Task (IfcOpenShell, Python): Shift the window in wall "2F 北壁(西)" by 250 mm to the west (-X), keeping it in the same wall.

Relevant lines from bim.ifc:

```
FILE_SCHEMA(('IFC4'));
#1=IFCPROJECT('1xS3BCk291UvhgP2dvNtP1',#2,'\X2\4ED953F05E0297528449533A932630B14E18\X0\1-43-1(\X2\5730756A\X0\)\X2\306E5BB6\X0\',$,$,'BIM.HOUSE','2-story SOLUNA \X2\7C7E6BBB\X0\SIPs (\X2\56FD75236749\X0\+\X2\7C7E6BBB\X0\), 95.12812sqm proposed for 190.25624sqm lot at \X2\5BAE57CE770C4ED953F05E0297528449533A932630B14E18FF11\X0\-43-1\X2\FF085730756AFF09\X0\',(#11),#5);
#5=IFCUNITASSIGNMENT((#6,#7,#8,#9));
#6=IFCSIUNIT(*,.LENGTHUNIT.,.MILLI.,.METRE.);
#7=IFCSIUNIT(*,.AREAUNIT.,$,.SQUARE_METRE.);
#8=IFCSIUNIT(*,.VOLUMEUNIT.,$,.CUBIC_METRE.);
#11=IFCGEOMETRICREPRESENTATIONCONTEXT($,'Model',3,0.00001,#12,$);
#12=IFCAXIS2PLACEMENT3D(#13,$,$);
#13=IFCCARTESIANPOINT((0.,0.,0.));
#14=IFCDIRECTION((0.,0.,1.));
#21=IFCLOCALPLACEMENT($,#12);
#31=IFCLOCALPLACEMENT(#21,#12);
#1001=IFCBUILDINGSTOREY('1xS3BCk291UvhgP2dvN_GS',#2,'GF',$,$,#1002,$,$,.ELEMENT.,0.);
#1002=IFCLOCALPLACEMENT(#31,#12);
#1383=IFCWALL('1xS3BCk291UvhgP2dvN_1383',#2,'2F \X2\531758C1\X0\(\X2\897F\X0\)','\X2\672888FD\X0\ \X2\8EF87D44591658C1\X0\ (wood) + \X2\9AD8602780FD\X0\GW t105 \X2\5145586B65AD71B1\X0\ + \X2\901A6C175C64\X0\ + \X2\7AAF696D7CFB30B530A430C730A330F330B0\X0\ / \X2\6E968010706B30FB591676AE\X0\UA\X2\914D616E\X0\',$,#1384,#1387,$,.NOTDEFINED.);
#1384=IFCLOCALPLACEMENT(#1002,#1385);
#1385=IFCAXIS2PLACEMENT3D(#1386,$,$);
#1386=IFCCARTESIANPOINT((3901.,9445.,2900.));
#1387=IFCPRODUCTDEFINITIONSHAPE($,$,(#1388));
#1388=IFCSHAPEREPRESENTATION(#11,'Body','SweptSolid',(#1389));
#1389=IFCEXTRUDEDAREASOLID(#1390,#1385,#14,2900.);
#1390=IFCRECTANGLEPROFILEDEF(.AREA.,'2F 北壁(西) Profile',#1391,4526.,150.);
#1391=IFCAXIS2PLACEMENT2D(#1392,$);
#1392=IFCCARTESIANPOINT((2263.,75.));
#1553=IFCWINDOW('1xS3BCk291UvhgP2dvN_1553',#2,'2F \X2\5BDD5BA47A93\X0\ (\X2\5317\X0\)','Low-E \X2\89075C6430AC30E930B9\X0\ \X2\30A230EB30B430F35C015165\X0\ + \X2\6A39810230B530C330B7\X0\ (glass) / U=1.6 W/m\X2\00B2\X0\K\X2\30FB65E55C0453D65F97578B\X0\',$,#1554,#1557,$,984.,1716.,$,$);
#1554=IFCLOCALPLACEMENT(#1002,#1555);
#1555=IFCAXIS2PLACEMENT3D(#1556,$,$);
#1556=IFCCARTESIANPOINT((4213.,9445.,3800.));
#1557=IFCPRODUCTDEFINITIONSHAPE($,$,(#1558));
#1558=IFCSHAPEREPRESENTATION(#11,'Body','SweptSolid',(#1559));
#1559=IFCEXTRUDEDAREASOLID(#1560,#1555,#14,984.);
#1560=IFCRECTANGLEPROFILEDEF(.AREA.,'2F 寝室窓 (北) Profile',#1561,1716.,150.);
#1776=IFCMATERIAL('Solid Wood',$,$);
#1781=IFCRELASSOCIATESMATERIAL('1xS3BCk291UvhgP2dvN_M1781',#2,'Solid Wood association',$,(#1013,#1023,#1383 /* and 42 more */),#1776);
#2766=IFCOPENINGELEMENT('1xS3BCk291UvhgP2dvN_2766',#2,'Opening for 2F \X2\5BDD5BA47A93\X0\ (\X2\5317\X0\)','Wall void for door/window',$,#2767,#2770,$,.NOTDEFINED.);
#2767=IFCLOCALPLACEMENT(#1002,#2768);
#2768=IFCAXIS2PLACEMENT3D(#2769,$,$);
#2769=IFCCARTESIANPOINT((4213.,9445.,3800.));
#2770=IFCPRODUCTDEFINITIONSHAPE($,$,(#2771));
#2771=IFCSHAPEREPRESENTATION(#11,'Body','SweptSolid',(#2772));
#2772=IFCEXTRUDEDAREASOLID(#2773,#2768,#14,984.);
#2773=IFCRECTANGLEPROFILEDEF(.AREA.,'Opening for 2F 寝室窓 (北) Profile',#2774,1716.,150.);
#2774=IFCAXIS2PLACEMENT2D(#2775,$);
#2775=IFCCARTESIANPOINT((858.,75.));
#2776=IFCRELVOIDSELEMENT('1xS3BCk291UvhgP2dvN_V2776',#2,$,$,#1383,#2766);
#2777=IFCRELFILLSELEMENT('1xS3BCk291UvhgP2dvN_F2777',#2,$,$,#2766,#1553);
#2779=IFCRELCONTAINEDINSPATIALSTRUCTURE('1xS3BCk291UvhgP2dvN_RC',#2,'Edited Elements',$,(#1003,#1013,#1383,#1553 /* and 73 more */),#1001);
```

```python
import ifcopenshell
import ifcopenshell.api.geometry
import ifcopenshell.util.placement
import ifcopenshell.util.unit

model = ifcopenshell.open("bim.ifc")
unit_scale = ifcopenshell.util.unit.calculate_unit_scale(model)

window = model.by_guid("1xS3BCk291UvhgP2dvN_1553")
opening = window.FillsVoids[0].RelatingOpeningElement
wall = opening.VoidsElements[0].RelatingBuildingElement

wall_matrix = ifcopenshell.util.placement.get_local_placement(wall.ObjectPlacement)
shift = wall_matrix[:3, 0] * -0.25 / unit_scale
before = ifcopenshell.util.placement.get_local_placement(window.ObjectPlacement)[:3, 3].copy()

# The window is not placed relative to its opening, so move both.
for product in (opening, window):
    matrix = ifcopenshell.util.placement.get_local_placement(product.ObjectPlacement)
    matrix[:3, 3] += shift
    ifcopenshell.api.geometry.edit_object_placement(model, product=product, matrix=matrix, is_si=False)

after = ifcopenshell.util.placement.get_local_placement(window.ObjectPlacement)[:3, 3]
print("window moved by", (after - before).round(3) + 0.0)

model.write("bim_v2.ifc")
```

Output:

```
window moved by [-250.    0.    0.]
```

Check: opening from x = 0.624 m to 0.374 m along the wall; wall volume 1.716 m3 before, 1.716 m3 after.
